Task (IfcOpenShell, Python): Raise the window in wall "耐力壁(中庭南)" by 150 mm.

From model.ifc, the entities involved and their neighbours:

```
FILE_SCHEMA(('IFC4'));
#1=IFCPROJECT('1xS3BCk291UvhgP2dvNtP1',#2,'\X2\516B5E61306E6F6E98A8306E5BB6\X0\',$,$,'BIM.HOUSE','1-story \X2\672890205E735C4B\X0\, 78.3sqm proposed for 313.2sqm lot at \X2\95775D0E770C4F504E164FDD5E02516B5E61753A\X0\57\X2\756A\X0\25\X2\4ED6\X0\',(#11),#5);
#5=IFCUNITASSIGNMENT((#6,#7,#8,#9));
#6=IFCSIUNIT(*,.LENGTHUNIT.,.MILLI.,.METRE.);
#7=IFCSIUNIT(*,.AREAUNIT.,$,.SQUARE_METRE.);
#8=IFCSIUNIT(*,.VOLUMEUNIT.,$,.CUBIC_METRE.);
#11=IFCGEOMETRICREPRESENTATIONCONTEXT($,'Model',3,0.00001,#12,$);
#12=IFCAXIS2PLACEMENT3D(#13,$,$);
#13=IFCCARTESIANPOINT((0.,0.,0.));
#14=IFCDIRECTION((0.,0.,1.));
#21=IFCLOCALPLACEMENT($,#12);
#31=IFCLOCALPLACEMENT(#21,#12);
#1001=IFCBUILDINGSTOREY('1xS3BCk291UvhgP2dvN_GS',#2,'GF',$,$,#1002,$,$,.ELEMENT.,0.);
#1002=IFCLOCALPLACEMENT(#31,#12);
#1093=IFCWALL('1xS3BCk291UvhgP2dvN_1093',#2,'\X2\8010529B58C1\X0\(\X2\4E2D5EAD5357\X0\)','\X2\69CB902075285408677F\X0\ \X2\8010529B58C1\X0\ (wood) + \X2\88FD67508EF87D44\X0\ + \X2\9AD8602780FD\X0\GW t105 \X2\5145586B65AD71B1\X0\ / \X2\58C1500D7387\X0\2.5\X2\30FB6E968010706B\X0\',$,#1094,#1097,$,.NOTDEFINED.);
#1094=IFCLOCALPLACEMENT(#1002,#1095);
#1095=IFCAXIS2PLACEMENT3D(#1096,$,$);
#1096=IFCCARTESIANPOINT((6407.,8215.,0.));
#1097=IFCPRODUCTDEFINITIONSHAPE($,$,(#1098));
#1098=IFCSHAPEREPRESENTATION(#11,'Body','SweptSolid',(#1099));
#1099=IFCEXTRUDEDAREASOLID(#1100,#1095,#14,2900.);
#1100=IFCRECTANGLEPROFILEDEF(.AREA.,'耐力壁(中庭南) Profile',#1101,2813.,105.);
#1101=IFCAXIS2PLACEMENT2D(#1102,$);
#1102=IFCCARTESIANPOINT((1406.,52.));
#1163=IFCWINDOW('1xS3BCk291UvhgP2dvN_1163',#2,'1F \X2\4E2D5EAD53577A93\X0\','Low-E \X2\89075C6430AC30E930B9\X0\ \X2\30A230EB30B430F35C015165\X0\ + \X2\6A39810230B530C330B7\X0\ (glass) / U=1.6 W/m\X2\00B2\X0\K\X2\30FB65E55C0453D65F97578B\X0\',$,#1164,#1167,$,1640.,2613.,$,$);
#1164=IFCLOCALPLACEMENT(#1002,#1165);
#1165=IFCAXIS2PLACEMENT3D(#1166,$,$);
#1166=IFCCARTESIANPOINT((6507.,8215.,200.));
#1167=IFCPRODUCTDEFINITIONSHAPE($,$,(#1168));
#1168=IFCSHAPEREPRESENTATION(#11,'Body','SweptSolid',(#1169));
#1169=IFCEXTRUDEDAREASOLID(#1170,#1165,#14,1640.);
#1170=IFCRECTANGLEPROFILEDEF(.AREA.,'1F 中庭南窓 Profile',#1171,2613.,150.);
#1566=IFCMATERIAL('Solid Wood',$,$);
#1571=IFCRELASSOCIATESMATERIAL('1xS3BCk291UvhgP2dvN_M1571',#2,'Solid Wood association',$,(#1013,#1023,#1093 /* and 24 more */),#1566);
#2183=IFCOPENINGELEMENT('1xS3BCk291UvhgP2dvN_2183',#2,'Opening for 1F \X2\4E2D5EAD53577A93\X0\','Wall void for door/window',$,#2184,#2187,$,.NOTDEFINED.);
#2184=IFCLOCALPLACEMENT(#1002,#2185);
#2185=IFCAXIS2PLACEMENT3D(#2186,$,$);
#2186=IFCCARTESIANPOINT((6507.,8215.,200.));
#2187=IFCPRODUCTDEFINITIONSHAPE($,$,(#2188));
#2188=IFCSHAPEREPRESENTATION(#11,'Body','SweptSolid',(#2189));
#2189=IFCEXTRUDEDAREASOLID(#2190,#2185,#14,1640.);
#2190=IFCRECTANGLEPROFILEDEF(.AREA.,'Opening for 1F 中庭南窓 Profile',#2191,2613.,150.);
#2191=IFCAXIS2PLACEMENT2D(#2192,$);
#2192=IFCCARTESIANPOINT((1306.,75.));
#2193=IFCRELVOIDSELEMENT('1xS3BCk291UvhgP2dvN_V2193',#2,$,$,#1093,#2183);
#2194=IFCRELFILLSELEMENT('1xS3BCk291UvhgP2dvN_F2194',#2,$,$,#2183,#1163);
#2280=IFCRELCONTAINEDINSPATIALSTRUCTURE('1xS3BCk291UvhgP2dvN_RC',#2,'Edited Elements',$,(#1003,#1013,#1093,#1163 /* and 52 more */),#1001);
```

```python
import numpy as np
import ifcopenshell
import ifcopenshell.api.geometry
import ifcopenshell.util.placement
import ifcopenshell.util.unit

model = ifcopenshell.open("model.ifc")
unit_scale = ifcopenshell.util.unit.calculate_unit_scale(model)

window = model.by_id(1163)
opening = window.FillsVoids[0].RelatingOpeningElement
dz = 0.15 / unit_scale

shift = np.array([0.0, 0.0, dz])
# The window is not placed relative to its opening, so move both.
for product in (opening, window):
    matrix = ifcopenshell.util.placement.get_local_placement(product.ObjectPlacement)
    matrix[:3, 3] += shift
    ifcopenshell.api.geometry.edit_object_placement(model, product=product, matrix=matrix, is_si=False)

print(f"moved by {dz * unit_scale:+.3f} m")

model.write("model_rev.ifc")
```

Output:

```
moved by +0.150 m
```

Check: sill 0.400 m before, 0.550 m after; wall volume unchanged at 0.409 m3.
